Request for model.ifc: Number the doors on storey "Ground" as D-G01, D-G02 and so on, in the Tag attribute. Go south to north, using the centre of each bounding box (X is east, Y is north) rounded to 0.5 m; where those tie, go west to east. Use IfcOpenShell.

First a look at what the model holds.

```python
import ifcopenshell
import ifcopenshell.util.element
import ifcopenshell.util.placement

model = ifcopenshell.open("model.ifc")
print(model.schema)
storey = next(s for s in model.by_type("IfcBuildingStorey") if s.Name == "Ground")
doors = [e for e in ifcopenshell.util.element.get_decomposition(storey) if e.is_a("IfcDoor")]
for e in sorted(doors, key=lambda e: e.id()):
    origin = ifcopenshell.util.placement.get_local_placement(e.ObjectPlacement)[:3, 3]
    print(e.id(), e.Tag, e.Name, origin.round(2) + 0.0, sep=" | ")
```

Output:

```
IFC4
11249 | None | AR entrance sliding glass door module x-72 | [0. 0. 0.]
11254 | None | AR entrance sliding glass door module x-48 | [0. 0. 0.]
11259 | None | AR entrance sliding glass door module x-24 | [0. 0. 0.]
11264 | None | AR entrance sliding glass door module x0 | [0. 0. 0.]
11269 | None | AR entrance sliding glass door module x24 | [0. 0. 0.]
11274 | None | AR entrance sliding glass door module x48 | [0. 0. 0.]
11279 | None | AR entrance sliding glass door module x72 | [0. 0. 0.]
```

```python
import ifcopenshell
import ifcopenshell.geom
import ifcopenshell.util.element
import ifcopenshell.util.shape

model = ifcopenshell.open("model.ifc")
settings = ifcopenshell.geom.settings()
settings.set("use-world-coords", True)


def centre(element):
    shape = ifcopenshell.geom.create_shape(settings, element)
    return ifcopenshell.util.shape.get_bbox_centroid(shape.geometry)


storey = next(s for s in model.by_type("IfcBuildingStorey") if s.Name == "Ground")
doors = [e for e in ifcopenshell.util.element.get_decomposition(storey) if e.is_a("IfcDoor")]

# Insertion points can sit at a corner or the storey origin, so sort by the geometry (in metres).
centres = {e: centre(e) for e in doors}
doors.sort(key=lambda e: (round(centres[e][1] / 0.5), centres[e][0]))

for i, e in enumerate(doors, start=1):
    number = f"D-G{i:02d}"
    e.Tag = number
    print(e.id(), number)

model.write("model_rev.ifc")
```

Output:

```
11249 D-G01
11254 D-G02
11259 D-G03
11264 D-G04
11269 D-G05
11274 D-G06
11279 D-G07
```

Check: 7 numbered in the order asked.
